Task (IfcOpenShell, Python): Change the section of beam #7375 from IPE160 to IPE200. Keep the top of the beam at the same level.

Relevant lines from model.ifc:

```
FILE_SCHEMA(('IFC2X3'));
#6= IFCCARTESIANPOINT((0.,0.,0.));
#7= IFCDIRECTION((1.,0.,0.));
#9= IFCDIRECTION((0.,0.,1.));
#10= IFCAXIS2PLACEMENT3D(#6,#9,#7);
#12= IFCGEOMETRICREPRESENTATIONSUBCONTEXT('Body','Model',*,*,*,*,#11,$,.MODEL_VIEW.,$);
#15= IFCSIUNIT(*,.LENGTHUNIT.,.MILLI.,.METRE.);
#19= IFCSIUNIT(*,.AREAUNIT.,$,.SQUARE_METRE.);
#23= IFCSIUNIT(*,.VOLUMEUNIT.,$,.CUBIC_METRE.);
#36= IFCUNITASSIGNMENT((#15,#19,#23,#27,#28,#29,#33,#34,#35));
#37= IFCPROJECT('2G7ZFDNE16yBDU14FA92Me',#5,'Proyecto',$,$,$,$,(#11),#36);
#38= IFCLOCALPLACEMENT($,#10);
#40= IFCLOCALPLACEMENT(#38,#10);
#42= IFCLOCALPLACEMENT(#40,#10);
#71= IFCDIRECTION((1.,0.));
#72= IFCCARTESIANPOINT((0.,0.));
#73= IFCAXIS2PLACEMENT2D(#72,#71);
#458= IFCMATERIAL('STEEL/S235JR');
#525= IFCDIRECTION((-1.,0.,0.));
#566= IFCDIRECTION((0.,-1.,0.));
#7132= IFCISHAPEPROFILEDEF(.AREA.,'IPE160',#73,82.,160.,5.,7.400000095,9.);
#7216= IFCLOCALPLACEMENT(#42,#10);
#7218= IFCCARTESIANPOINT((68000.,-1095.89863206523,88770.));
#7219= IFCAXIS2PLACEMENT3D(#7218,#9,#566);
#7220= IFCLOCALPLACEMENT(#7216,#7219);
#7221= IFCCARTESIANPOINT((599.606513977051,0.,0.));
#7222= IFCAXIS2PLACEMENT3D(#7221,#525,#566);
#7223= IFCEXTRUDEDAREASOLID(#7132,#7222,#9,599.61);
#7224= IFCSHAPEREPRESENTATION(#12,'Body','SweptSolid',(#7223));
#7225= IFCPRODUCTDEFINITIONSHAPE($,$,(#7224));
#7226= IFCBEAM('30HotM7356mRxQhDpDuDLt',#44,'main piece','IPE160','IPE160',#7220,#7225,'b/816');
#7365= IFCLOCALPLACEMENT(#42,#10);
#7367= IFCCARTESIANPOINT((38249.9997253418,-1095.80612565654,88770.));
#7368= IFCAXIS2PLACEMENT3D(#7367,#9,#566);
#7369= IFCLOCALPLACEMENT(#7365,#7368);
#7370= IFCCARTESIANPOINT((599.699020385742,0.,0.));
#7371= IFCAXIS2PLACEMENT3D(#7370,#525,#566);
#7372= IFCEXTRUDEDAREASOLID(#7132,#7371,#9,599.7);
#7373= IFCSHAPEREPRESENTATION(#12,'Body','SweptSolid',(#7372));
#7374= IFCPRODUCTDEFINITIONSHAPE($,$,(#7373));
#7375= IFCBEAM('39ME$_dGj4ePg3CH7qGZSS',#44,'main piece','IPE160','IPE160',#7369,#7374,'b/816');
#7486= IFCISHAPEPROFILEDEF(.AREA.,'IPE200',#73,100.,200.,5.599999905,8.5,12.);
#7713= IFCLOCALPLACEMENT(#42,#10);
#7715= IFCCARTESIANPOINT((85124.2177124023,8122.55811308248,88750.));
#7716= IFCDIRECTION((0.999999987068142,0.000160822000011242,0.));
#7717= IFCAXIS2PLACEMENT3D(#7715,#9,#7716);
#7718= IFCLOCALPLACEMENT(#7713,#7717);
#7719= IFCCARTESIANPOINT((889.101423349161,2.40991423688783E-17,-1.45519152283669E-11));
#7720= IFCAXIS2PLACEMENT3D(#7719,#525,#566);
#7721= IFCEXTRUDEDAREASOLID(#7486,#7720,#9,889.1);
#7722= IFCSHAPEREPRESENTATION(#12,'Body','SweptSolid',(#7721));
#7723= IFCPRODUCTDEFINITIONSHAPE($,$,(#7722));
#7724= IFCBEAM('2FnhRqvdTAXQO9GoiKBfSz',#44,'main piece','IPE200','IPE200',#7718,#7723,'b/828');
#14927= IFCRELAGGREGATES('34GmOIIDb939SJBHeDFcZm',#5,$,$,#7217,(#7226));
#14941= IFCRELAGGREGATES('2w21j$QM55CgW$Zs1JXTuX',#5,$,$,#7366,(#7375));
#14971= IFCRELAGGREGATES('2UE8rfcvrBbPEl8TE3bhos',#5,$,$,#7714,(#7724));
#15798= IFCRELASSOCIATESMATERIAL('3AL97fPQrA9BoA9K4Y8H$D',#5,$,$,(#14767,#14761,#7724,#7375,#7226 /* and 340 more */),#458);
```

```python
import ifcopenshell
import ifcopenshell.util.element
import ifcopenshell.util.representation

model = ifcopenshell.open("model.ifc")

member = model.by_guid("39ME$_dGj4ePg3CH7qGZSS")
source = next(p for p in model.by_type("IfcIShapeProfileDef") if p.ProfileName == "IPE200")

body = ifcopenshell.util.representation.get_representation(member, "Model", "Body")
solid = body.Items[0]
old_profile = solid.SweptArea

# Copy the section's sizes but keep this member's own profile position.
profile = ifcopenshell.util.element.copy(model, source)
# Profiles are centred, so shift by half the change in depth to hold the top.
shift = (old_profile.OverallDepth - profile.OverallDepth) / 2
x, y = old_profile.Position.Location.Coordinates
up = (0.0, 1.0)  # upwards, in the solid's own plane
location = model.createIfcCartesianPoint((x + up[0] * shift, y + up[1] * shift))
profile.Position = model.createIfcAxis2Placement2D(location, old_profile.Position.RefDirection)
solid.SweptArea = profile
if not model.get_total_inverses(old_profile):
    ifcopenshell.util.element.remove_deep2(model, old_profile)
member.Description = member.Description.replace("IPE160", "IPE200")
member.ObjectType = member.ObjectType.replace("IPE160", "IPE200")

print(solid.SweptArea)

model.write("model_edited.ifc")
```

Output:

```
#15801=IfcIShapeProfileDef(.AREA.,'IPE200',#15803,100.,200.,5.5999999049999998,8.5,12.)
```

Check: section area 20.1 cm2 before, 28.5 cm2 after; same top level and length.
